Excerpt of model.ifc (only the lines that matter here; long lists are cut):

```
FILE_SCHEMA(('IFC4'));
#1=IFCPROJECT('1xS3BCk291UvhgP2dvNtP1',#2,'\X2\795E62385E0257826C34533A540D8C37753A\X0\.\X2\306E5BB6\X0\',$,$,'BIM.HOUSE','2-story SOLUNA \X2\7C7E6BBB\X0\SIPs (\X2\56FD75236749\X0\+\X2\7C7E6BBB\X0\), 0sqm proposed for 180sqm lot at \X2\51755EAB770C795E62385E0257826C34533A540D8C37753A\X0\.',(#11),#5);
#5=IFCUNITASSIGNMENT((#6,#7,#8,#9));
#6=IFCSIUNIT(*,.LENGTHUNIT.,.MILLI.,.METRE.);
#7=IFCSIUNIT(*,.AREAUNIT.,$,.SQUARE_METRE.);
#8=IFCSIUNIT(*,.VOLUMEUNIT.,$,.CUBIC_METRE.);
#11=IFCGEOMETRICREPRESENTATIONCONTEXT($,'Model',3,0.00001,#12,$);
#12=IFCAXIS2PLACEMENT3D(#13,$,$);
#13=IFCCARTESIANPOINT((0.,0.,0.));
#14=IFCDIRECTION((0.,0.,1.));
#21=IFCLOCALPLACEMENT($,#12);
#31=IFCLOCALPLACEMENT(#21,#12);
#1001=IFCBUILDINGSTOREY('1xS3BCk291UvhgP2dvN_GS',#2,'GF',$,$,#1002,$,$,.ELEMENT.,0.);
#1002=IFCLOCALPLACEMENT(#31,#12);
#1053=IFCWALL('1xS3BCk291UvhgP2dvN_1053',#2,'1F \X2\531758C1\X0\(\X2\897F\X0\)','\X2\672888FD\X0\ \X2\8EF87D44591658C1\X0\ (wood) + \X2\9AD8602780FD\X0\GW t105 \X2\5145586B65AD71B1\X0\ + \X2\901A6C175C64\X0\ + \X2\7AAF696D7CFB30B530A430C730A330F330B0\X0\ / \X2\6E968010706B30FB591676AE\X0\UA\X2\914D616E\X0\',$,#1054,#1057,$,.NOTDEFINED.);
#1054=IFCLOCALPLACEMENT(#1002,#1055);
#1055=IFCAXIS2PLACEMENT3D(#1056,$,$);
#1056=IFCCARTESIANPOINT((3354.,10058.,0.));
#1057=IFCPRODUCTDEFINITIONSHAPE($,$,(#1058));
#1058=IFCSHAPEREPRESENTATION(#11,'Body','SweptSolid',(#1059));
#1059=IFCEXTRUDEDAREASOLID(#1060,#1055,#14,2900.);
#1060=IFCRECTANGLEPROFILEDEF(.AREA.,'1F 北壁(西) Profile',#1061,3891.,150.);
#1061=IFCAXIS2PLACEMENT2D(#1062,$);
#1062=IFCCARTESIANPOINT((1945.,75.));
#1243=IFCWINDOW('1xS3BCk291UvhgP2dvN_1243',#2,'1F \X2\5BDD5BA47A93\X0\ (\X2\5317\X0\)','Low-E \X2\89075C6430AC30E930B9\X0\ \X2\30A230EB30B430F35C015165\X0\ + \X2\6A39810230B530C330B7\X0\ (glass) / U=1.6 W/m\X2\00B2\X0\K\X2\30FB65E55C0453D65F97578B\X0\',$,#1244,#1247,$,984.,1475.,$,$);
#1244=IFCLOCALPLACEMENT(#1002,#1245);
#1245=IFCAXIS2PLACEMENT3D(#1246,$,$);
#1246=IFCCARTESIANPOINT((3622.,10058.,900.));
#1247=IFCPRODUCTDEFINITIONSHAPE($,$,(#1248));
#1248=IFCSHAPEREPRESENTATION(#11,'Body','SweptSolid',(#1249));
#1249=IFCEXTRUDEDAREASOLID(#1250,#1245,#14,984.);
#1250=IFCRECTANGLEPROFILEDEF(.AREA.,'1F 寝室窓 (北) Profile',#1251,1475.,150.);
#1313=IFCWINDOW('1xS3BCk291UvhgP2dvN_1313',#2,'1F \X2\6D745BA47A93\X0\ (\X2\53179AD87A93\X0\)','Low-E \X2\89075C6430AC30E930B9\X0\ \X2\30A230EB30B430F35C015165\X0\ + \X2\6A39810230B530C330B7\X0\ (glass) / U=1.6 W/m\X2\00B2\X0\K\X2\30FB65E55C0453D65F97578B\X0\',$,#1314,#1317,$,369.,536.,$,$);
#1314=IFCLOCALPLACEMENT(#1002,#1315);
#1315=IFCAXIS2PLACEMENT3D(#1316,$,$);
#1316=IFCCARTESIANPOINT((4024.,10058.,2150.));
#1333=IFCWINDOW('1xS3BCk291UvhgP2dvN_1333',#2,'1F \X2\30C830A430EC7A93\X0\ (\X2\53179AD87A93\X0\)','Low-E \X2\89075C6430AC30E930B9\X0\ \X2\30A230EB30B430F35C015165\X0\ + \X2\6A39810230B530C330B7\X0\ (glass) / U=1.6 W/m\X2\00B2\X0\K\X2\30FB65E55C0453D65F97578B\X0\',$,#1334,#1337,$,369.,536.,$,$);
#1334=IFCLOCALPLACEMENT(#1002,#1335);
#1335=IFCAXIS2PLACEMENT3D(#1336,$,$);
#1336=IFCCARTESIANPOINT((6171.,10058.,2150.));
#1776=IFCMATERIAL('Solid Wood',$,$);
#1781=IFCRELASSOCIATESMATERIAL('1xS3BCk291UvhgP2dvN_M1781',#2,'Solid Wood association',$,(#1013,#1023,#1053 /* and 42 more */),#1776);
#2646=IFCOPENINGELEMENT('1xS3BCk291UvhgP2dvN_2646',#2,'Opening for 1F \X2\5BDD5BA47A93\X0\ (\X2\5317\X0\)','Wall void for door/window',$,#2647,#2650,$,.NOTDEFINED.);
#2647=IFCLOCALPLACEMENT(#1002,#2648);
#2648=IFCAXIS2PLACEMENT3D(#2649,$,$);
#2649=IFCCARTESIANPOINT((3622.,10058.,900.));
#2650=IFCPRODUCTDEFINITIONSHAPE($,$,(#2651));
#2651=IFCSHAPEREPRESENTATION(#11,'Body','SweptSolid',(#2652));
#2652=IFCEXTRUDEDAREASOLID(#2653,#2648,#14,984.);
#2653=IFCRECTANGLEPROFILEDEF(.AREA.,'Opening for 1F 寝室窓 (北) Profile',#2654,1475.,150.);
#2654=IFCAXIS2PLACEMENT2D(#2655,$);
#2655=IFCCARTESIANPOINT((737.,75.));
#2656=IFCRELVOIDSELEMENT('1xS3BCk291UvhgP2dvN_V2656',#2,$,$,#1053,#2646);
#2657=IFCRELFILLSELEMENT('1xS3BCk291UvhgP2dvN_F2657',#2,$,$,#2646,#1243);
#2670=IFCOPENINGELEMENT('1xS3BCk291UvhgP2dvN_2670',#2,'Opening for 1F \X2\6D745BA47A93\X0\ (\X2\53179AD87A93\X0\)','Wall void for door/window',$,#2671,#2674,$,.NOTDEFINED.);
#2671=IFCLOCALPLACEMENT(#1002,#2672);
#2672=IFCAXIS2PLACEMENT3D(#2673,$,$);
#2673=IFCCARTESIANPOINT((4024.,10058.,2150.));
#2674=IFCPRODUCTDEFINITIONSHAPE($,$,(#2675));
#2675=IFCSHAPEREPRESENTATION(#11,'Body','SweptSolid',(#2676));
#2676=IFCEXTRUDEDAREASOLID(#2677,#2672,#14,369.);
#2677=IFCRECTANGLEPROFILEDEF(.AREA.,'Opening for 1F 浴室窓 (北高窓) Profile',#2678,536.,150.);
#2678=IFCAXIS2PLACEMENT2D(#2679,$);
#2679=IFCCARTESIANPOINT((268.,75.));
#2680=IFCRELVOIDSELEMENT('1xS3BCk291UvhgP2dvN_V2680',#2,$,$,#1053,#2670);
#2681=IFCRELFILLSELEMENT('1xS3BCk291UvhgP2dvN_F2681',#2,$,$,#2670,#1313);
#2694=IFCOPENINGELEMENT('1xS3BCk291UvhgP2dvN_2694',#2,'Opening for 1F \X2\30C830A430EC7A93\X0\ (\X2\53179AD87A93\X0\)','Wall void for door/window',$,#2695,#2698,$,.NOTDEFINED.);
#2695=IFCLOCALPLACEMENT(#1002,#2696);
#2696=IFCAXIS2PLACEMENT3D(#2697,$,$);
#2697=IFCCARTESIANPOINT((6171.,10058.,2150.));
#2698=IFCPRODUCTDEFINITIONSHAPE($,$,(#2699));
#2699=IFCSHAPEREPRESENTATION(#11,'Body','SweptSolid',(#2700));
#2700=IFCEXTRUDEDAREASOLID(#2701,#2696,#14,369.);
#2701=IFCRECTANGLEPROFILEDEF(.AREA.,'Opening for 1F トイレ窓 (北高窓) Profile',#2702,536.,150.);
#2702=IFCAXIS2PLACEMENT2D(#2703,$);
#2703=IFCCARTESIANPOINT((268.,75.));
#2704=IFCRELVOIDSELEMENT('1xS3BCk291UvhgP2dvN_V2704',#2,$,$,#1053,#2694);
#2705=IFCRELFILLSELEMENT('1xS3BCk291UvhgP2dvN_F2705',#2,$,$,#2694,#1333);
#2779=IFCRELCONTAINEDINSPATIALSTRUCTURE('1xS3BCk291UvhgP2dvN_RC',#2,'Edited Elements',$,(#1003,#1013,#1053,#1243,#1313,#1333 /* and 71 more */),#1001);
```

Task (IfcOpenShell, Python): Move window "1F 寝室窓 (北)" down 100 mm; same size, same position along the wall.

```python
import numpy as np
import ifcopenshell
import ifcopenshell.api.geometry
import ifcopenshell.util.placement
import ifcopenshell.util.unit

model = ifcopenshell.open("model.ifc")
unit_scale = ifcopenshell.util.unit.calculate_unit_scale(model)

window = model.by_guid("1xS3BCk291UvhgP2dvN_1243")
opening = window.FillsVoids[0].RelatingOpeningElement
dz = -100.0

shift = np.array([0.0, 0.0, dz])
# The window is not placed relative to its opening, so move both.
for product in (opening, window):
    matrix = ifcopenshell.util.placement.get_local_placement(product.ObjectPlacement)
    matrix[:3, 3] += shift
    ifcopenshell.api.geometry.edit_object_placement(model, product=product, matrix=matrix, is_si=False)

print(f"moved by {dz * unit_scale:+.3f} m")

model.write("model_edited.ifc")
```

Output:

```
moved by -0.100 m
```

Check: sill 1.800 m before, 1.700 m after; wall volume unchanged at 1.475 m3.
